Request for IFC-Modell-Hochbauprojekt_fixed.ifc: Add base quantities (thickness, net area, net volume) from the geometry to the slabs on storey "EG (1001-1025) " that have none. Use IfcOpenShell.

First a look at what the model holds.

```python
import ifcopenshell
import ifcopenshell.util.element
import ifcopenshell.util.unit

model = ifcopenshell.open("IFC-Modell-Hochbauprojekt_fixed.ifc")
print(model.schema)
for unit_type in ("LENGTHUNIT", "AREAUNIT", "VOLUMEUNIT"):
    print(unit_type, ifcopenshell.util.unit.calculate_unit_scale(model, unit_type))
storey = next(s for s in model.by_type("IfcBuildingStorey") if s.Name == "EG (1001-1025) ")
slabs = [e for e in ifcopenshell.util.element.get_decomposition(storey) if e.is_a("IfcSlab")]
for e in sorted(slabs, key=lambda e: e.id()):
    print(e.id(), e.is_a(), e.Name, list(ifcopenshell.util.element.get_psets(e, qtos_only=True)), sep=" | ")
```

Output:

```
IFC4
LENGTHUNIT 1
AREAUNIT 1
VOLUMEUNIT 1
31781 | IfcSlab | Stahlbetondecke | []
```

```python
import ifcopenshell
import ifcopenshell.api.pset
import ifcopenshell.geom
import ifcopenshell.util.element
import ifcopenshell.util.shape
import ifcopenshell.util.unit

model = ifcopenshell.open("IFC-Modell-Hochbauprojekt_fixed.ifc")
unit_scale = ifcopenshell.util.unit.calculate_unit_scale(model)
area_scale = ifcopenshell.util.unit.calculate_unit_scale(model, "AREAUNIT")
volume_scale = ifcopenshell.util.unit.calculate_unit_scale(model, "VOLUMEUNIT")
settings = ifcopenshell.geom.settings()

storey = next(s for s in model.by_type("IfcBuildingStorey") if s.Name == "EG (1001-1025) ")
slabs = [e for e in ifcopenshell.util.element.get_decomposition(storey) if e.is_a("IfcSlab")]

for e in sorted(slabs, key=lambda e: e.id()):
    if ifcopenshell.util.element.get_psets(e, qtos_only=True, should_inherit=False):
        continue
    # Geometry comes back in metres, in the element's own axes.
    shape = ifcopenshell.geom.create_shape(settings, e)
    values = {
        "Width": ifcopenshell.util.shape.get_z(shape.geometry) / unit_scale,
        "NetArea": ifcopenshell.util.shape.get_footprint_area(shape.geometry) / area_scale,
        "NetVolume": ifcopenshell.util.shape.get_volume(shape.geometry) / volume_scale,
    }
    qto = ifcopenshell.api.pset.add_qto(model, product=e, name="Qto_SlabBaseQuantities")
    ifcopenshell.api.pset.edit_qto(model, qto=qto, properties=values)
    print(e.id(), {k: round(v, 3) for k, v in values.items()})

model.write("IFC-Modell-Hochbauprojekt_fixed_edited.ifc")
```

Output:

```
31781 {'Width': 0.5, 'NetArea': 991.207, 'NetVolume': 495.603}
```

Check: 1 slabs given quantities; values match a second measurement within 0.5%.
